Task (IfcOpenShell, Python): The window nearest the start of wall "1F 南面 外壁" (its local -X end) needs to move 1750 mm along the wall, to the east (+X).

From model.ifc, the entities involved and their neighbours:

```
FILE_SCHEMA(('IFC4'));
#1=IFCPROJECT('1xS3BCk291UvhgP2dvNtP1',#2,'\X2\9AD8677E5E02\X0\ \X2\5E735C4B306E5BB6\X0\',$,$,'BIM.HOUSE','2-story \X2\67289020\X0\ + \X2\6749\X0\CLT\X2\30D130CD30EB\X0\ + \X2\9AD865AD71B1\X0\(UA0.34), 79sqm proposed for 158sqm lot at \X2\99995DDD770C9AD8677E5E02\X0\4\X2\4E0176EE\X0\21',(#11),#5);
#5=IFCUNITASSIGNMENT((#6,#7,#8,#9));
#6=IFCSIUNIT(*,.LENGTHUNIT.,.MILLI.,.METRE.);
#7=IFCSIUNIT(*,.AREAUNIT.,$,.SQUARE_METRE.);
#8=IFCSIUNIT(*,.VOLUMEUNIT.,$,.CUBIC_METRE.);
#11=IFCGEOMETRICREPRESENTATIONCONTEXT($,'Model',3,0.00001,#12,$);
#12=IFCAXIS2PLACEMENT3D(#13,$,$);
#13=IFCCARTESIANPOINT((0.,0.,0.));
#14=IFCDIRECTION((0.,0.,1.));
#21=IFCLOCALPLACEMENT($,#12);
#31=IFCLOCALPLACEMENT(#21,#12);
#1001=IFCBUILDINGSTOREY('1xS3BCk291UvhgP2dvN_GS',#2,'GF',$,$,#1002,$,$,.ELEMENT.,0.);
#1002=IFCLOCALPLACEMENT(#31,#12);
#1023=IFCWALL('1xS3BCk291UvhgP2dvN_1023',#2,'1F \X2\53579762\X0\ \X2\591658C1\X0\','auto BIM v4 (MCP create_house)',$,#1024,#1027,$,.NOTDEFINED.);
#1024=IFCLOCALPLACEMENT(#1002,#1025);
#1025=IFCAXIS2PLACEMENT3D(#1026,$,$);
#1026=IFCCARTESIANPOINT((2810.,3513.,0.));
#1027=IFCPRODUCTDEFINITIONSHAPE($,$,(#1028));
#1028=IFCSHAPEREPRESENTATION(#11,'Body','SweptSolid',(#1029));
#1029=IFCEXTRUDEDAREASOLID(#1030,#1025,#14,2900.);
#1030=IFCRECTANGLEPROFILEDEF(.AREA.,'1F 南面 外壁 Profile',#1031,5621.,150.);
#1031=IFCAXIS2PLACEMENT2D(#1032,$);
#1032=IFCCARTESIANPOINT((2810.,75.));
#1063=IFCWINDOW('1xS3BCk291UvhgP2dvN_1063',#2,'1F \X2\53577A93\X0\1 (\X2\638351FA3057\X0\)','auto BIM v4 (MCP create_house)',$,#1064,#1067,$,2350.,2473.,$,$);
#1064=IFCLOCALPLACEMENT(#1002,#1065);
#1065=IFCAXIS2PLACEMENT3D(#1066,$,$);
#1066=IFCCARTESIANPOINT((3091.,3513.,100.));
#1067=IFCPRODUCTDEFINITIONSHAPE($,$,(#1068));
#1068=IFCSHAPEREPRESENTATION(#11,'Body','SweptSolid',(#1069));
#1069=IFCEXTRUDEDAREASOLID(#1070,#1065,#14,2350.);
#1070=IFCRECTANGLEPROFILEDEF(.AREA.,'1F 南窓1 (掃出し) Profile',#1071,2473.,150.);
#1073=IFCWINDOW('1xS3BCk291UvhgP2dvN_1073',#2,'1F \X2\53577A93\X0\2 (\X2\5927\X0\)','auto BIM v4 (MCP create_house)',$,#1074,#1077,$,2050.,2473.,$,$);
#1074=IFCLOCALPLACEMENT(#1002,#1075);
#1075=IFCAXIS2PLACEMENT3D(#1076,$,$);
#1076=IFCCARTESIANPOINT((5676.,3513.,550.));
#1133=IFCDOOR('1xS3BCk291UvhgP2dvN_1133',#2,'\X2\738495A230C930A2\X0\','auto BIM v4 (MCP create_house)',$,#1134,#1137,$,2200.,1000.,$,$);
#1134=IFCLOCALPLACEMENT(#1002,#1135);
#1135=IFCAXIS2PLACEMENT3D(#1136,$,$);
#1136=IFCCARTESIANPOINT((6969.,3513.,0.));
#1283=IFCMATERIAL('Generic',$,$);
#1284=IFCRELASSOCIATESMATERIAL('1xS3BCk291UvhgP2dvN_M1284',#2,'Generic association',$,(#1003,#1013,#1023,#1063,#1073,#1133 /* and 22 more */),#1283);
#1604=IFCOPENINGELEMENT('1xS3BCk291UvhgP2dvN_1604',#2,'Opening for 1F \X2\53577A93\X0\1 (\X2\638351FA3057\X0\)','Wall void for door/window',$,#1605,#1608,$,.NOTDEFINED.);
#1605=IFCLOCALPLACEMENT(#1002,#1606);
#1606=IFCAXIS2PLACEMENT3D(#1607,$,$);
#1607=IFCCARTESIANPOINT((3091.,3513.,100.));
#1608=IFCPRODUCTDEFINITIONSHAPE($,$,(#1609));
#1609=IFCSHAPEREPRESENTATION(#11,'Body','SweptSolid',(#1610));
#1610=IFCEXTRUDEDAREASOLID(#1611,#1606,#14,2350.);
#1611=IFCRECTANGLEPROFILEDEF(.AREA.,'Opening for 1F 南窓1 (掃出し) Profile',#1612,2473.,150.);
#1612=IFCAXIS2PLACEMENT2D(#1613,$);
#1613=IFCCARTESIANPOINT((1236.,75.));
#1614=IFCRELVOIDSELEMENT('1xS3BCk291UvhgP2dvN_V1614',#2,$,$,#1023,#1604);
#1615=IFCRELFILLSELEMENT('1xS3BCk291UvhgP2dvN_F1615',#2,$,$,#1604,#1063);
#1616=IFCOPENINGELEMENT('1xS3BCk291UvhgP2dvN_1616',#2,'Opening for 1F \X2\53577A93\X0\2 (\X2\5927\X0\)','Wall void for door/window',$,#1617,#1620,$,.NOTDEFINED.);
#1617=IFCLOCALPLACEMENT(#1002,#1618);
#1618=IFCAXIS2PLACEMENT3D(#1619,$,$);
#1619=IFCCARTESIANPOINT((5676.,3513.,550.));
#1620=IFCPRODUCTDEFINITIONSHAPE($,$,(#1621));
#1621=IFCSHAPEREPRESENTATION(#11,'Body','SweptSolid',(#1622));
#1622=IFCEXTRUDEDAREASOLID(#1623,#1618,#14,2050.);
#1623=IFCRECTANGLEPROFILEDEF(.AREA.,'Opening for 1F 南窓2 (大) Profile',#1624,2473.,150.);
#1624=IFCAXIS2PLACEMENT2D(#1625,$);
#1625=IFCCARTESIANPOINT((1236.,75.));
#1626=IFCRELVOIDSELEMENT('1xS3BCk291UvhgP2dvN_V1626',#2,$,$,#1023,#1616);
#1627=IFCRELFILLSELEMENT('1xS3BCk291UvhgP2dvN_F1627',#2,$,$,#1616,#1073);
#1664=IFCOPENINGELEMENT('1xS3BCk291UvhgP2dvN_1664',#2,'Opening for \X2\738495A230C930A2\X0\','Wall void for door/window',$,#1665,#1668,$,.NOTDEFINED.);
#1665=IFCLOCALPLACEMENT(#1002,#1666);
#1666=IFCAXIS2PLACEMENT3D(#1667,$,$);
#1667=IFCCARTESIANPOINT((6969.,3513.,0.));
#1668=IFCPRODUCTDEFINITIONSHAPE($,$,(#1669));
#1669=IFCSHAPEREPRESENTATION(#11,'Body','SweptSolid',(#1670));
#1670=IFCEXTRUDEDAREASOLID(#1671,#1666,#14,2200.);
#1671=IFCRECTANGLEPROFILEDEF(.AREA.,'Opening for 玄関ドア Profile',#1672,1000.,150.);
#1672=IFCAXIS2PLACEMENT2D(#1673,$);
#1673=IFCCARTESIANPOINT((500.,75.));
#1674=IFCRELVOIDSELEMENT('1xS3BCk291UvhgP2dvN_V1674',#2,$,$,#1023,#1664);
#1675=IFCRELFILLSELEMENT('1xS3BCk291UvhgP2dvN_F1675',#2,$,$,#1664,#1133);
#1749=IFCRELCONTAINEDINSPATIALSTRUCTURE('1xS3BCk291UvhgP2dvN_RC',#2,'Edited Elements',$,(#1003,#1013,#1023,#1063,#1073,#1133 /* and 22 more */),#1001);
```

```python
import ifcopenshell
import ifcopenshell.api.geometry
import ifcopenshell.util.placement

model = ifcopenshell.open("model.ifc")

window = model.by_id(1063)
opening = window.FillsVoids[0].RelatingOpeningElement
wall = opening.VoidsElements[0].RelatingBuildingElement

wall_matrix = ifcopenshell.util.placement.get_local_placement(wall.ObjectPlacement)
shift = wall_matrix[:3, 0] * 1750.0
before = ifcopenshell.util.placement.get_local_placement(window.ObjectPlacement)[:3, 3].copy()

# The window is not placed relative to its opening, so move both.
for product in (opening, window):
    matrix = ifcopenshell.util.placement.get_local_placement(product.ObjectPlacement)
    matrix[:3, 3] += shift
    ifcopenshell.api.geometry.edit_object_placement(model, product=product, matrix=matrix, is_si=False)

after = ifcopenshell.util.placement.get_local_placement(window.ObjectPlacement)[:3, 3]
print("window moved by", (after - before).round(3) + 0.0)

model.write("model_rev.ifc")
```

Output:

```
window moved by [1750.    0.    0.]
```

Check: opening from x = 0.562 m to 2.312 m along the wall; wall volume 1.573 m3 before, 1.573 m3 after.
